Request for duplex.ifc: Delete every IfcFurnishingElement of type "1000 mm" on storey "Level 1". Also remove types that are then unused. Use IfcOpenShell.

First a look at what the model holds.

```python
import ifcopenshell
import ifcopenshell.util.element

model = ifcopenshell.open("duplex.ifc")
print(model.schema)
storey = next(s for s in model.by_type("IfcBuildingStorey") if s.Name == "Level 1")
furniture = [e for e in ifcopenshell.util.element.get_decomposition(storey) if e.is_a("IfcFurnishingElement")]
seen = {}
for e in furniture:
    element_type = ifcopenshell.util.element.get_type(e)
    name = element_type.Name if element_type not in (None, e) else None
    seen[name] = seen.get(name, 0) + 1
for name, count in sorted(seen.items(), key=str):
    print(count, "x", name)
```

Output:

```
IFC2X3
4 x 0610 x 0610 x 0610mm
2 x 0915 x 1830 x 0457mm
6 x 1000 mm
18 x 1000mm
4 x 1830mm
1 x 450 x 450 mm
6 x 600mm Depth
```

```python
import ifcopenshell
import ifcopenshell.api.root
import ifcopenshell.util.element

model = ifcopenshell.open("duplex.ifc")

storey = next(s for s in model.by_type("IfcBuildingStorey") if s.Name == "Level 1")
furniture = [e for e in ifcopenshell.util.element.get_decomposition(storey) if e.is_a("IfcFurnishingElement")]
targets = [e for e in furniture if (t := ifcopenshell.util.element.get_type(e)) not in (None, e) and t.Name == "1000 mm"]
types = {ifcopenshell.util.element.get_type(e) for e in targets} - {None, *targets}

for e in targets:
    ifcopenshell.api.root.remove_product(model, product=e)
print(len(targets), "removed")

unused = [t for t in types if not ifcopenshell.util.element.get_types(t)]
for t in unused:
    ifcopenshell.api.root.remove_product(model, product=t)
print(len(unused), "unused types removed")

model.write("duplex_v2.ifc")
```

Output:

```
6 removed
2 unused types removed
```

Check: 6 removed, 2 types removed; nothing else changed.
